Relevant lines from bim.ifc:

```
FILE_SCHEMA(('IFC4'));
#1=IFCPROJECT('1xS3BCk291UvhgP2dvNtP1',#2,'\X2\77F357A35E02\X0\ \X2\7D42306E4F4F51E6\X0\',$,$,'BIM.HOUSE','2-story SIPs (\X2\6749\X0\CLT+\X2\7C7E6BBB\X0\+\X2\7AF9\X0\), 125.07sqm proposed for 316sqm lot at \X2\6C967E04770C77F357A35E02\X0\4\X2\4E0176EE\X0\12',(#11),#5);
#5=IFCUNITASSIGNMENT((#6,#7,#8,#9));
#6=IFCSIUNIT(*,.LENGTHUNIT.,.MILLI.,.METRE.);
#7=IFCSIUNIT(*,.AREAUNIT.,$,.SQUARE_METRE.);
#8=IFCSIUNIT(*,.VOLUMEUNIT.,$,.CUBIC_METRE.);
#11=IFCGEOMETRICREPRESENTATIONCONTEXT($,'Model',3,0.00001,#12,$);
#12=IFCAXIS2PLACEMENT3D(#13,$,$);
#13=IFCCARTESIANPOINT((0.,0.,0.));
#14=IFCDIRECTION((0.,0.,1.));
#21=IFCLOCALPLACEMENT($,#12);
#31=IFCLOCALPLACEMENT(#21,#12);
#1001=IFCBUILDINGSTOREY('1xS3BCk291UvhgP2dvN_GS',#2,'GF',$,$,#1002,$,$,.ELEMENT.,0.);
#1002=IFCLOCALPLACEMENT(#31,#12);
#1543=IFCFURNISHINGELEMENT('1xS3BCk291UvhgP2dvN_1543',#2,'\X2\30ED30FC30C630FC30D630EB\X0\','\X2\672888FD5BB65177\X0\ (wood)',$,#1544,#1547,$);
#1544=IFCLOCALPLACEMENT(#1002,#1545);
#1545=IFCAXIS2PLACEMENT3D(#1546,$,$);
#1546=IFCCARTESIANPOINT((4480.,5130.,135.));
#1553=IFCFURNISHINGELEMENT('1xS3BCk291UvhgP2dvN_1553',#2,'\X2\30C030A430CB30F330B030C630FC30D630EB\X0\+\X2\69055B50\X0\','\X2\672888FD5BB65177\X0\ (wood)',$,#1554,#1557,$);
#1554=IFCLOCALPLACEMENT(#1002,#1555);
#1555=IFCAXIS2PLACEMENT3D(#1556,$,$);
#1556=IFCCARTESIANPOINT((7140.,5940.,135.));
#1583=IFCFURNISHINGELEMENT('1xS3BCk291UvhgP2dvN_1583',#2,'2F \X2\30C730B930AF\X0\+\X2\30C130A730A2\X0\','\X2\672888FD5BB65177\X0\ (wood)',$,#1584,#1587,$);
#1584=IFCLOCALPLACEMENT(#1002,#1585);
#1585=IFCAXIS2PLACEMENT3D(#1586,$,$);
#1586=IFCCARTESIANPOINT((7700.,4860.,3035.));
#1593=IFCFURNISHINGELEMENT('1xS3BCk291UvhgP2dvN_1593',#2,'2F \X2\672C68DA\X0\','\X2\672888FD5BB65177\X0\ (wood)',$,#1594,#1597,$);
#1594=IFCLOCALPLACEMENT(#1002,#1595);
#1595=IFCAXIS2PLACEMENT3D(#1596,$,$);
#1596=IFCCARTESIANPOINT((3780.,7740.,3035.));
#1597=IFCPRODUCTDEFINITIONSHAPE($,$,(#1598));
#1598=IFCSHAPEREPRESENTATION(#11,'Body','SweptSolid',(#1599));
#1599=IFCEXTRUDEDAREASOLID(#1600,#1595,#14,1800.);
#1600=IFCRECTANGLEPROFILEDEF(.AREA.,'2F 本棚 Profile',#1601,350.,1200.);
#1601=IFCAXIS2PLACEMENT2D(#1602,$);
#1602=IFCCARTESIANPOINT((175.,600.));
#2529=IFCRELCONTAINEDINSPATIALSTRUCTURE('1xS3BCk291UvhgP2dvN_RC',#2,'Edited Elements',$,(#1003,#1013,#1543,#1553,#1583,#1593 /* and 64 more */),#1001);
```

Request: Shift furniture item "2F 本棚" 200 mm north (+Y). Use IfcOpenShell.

```python
import ifcopenshell
import ifcopenshell.api.geometry
import ifcopenshell.util.placement

model = ifcopenshell.open("bim.ifc")

item = model.by_guid("1xS3BCk291UvhgP2dvN_1593")
matrix = ifcopenshell.util.placement.get_local_placement(item.ObjectPlacement)
matrix[1, 3] += 200.0
ifcopenshell.api.geometry.edit_object_placement(model, product=item, matrix=matrix, is_si=False)

print(ifcopenshell.util.placement.get_local_placement(item.ObjectPlacement).round(3) + 0.0)

model.write("bim-out.ifc")
```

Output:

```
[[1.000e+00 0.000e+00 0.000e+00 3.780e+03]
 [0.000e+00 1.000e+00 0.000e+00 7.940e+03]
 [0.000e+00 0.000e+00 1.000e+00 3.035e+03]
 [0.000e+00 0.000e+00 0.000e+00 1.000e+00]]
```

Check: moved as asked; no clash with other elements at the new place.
